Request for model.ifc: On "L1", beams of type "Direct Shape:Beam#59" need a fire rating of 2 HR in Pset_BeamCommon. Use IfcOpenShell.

First a look at what the model holds.

```python
import ifcopenshell
import ifcopenshell.util.element

model = ifcopenshell.open("model.ifc")
print(model.schema)
storey = next(s for s in model.by_type("IfcBuildingStorey") if s.Name == "L1")
beams = [e for e in ifcopenshell.util.element.get_decomposition(storey) if e.is_a("IfcBeam")]
seen = {}
for e in beams:
    element_type = ifcopenshell.util.element.get_type(e)
    key = (element_type.Name if element_type != e and element_type else None, ifcopenshell.util.element.get_pset(e, "Pset_BeamCommon", "FireRating"))
    seen[key] = seen.get(key, 0) + 1
for (name, value), count in sorted(seen.items(), key=str):
    print(count, "x", name, "|", value)
```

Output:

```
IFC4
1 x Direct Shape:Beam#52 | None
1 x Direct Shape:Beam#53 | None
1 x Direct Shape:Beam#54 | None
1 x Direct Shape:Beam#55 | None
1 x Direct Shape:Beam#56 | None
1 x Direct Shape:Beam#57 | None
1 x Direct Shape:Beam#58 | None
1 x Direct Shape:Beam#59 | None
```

```python
import ifcopenshell
import ifcopenshell.api.pset
import ifcopenshell.util.element

model = ifcopenshell.open("model.ifc")

storey = next(s for s in model.by_type("IfcBuildingStorey") if s.Name == "L1")
beams = [e for e in ifcopenshell.util.element.get_decomposition(storey) if e.is_a("IfcBeam")]

count = 0
for e in beams:
    element_type = ifcopenshell.util.element.get_type(e)
    if element_type in (None, e) or element_type.Name != "Direct Shape:Beam#59":
        continue
    # add_pset returns the element's existing set when there is one.
    pset = ifcopenshell.api.pset.add_pset(model, product=e, name="Pset_BeamCommon")
    ifcopenshell.api.pset.edit_pset(model, pset=pset, properties={"FireRating": "2 HR"})
    count += 1

print(count, "beams updated")

model.write("model_updated.ifc")
```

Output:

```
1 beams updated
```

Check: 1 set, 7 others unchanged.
